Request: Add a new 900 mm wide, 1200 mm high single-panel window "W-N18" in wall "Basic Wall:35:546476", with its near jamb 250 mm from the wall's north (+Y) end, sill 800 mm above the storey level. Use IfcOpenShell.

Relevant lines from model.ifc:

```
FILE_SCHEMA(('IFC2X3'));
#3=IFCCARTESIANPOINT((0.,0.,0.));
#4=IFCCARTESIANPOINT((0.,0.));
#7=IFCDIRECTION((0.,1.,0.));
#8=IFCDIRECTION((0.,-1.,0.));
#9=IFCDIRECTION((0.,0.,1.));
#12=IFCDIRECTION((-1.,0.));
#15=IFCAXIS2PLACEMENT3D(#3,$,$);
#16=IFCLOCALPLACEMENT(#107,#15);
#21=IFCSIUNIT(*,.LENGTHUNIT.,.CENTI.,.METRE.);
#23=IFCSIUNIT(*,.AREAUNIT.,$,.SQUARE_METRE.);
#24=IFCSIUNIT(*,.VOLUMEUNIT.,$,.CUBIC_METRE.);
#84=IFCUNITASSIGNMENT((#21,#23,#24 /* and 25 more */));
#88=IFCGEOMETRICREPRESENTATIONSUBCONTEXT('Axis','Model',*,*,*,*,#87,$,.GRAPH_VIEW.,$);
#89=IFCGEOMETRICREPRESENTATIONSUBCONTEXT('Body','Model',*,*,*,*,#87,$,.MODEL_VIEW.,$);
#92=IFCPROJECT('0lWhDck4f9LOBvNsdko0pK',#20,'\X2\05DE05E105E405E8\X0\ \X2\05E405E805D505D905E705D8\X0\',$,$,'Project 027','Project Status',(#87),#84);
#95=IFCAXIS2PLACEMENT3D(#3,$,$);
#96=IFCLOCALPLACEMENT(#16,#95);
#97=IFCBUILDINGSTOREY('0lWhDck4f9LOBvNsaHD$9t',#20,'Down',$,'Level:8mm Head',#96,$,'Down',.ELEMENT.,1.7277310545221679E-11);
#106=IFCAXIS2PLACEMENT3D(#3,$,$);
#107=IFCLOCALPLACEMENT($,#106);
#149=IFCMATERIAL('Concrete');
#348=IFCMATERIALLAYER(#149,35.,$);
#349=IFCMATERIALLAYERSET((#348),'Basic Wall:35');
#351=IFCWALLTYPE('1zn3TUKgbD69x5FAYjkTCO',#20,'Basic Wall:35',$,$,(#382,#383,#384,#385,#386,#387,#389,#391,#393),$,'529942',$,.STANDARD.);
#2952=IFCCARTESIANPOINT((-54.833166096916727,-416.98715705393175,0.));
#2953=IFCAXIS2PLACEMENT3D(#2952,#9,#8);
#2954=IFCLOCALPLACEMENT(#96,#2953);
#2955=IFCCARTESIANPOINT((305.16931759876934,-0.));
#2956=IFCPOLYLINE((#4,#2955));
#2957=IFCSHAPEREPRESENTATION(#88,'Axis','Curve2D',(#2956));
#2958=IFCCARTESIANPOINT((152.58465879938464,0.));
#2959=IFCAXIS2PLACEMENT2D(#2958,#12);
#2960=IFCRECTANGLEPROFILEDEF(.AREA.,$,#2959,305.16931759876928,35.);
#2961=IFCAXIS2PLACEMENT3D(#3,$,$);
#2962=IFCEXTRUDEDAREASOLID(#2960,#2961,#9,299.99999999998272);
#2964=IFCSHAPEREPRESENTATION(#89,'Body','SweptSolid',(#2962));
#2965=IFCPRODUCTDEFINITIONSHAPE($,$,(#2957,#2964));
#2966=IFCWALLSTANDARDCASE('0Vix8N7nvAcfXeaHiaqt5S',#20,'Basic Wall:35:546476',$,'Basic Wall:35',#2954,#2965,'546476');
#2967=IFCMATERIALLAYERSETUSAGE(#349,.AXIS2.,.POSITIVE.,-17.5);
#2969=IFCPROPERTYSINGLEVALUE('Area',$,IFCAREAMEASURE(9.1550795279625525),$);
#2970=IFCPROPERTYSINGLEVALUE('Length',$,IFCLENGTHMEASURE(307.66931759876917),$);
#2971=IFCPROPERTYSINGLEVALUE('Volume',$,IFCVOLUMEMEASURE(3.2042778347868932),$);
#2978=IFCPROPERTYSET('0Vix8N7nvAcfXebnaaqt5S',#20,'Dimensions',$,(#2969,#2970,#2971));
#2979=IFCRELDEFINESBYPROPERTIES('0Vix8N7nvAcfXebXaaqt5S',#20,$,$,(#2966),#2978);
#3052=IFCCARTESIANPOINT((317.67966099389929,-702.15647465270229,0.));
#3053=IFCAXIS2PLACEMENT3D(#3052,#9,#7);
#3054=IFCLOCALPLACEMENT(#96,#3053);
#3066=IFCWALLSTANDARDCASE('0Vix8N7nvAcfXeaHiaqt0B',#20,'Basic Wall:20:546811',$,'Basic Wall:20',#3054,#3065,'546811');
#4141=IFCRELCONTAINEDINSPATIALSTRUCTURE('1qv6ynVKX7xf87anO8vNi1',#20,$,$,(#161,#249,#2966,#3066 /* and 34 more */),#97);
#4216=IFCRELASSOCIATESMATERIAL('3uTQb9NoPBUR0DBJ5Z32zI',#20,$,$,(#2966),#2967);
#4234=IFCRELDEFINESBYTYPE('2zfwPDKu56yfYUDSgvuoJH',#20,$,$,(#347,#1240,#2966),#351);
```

```python
import numpy as np
import ifcopenshell
import ifcopenshell.api.feature
import ifcopenshell.api.geometry
import ifcopenshell.api.pset
import ifcopenshell.api.root
import ifcopenshell.api.spatial
import ifcopenshell.api.type
import ifcopenshell.geom
import ifcopenshell.util.element
import ifcopenshell.util.placement
import ifcopenshell.util.representation
import ifcopenshell.util.shape
import ifcopenshell.util.unit

model = ifcopenshell.open("model.ifc")
unit_scale = ifcopenshell.util.unit.calculate_unit_scale(model)
area_scale = ifcopenshell.util.unit.calculate_unit_scale(model, "AREAUNIT")
volume_scale = ifcopenshell.util.unit.calculate_unit_scale(model, "VOLUMEUNIT")
settings = ifcopenshell.geom.settings()


def volume(element):
    """Net volume in cubic metres, openings subtracted."""
    shape = ifcopenshell.geom.create_shape(settings, element)
    return ifcopenshell.util.shape.get_volume(shape.geometry)


wall = model.by_id(2966)
storey = ifcopenshell.util.element.get_container(wall, ifc_class="IfcBuildingStorey")
context = ifcopenshell.util.representation.get_context(model, "Model", "Body", "MODEL_VIEW")
before = volume(wall)

width, height, from_end, sill = 0.9, 1.2, 0.25, 0.8  # metres

# The wall runs along its own X axis, and the end named is its -X end.
wall_shape = ifcopenshell.geom.create_shape(settings, wall)
x, y, z = ifcopenshell.util.shape.get_vertices(wall_shape.geometry).T
start = x.min() + from_end
face, thickness = float(y.min()), float(y.max() - y.min())
wall_matrix = ifcopenshell.util.placement.get_local_placement(wall.ObjectPlacement)
level = ifcopenshell.util.placement.get_local_placement(storey.ObjectPlacement)[2, 3]


def in_wall(x, y):
    """Placement at x, y metres in the wall's axes, at sill height."""
    matrix = wall_matrix.copy()
    matrix[:, 3] = wall_matrix @ np.array([x / unit_scale, y / unit_scale, 0.0, 1.0])
    matrix[2, 3] = level + sill / unit_scale
    return matrix


# Opening: a box that overshoots both wall faces by 50 mm.
opening = ifcopenshell.api.root.create_entity(model, ifc_class="IfcOpeningElement")
box = ifcopenshell.api.geometry.add_wall_representation(
    model, context=context, length=width, height=height, thickness=thickness + 0.1
)
ifcopenshell.api.geometry.assign_representation(model, product=opening, representation=box)
ifcopenshell.api.geometry.edit_object_placement(model, product=opening, matrix=in_wall(start, face - 0.05), is_si=False)
ifcopenshell.api.feature.add_feature(model, feature=opening, element=wall)

window = ifcopenshell.api.root.create_entity(model, ifc_class="IfcWindow", name="W-N18")
window.OverallWidth, window.OverallHeight = width / unit_scale, height / unit_scale
body = ifcopenshell.api.geometry.add_window_representation(
    model,
    context=context,
    overall_width=window.OverallWidth,
    overall_height=window.OverallHeight,
    partition_type="SINGLE_PANEL",
)
ifcopenshell.api.geometry.assign_representation(model, product=window, representation=body)
ifcopenshell.api.spatial.assign_container(model, products=[window], relating_structure=storey)
fills = ifcopenshell.api.feature.add_filling(model, opening=opening, element=window)
fills.OwnerHistory = window.OwnerHistory  # required in IFC2X3

# IFC2X3 keeps the operation on the window style.
style = ifcopenshell.api.root.create_entity(model, ifc_class="IfcWindowStyle", name="W-N18")
style.OperationType, style.ConstructionType = "SINGLE_PANEL", "NOTDEFINED"
style.ParameterTakesPrecedence = style.Sizeable = False
ifcopenshell.api.type.assign_type(model, related_objects=[window], relating_type=style)

# Centre the window in the wall's thickness.
ifcopenshell.api.geometry.edit_object_placement(model, product=window, matrix=in_wall(start, face), is_si=False)
window_shape = ifcopenshell.geom.create_shape(settings, window)
depth = ifcopenshell.util.shape.get_vertices(window_shape.geometry)[:, 1]
offset = face + thickness / 2 - (depth.min() + depth.max()) / 2
ifcopenshell.api.geometry.edit_object_placement(model, product=window, matrix=in_wall(start, offset), is_si=False)

after = volume(wall)

# Update the wall's stored quantities.
pset = model.by_id(ifcopenshell.util.element.get_pset(wall, "Dimensions", should_inherit=False)["id"])
ifcopenshell.api.pset.edit_pset(model, pset=pset, properties={
    "Area": model.create_entity("IfcAreaMeasure", after / thickness / area_scale),
    "Volume": model.create_entity("IfcVolumeMeasure", after / volume_scale),
})

print(f"wall volume {before:.3f} -> {after:.3f} m3")

model.write("model_rev.ifc")
```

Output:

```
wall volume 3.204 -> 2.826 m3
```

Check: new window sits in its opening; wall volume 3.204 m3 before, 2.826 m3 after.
